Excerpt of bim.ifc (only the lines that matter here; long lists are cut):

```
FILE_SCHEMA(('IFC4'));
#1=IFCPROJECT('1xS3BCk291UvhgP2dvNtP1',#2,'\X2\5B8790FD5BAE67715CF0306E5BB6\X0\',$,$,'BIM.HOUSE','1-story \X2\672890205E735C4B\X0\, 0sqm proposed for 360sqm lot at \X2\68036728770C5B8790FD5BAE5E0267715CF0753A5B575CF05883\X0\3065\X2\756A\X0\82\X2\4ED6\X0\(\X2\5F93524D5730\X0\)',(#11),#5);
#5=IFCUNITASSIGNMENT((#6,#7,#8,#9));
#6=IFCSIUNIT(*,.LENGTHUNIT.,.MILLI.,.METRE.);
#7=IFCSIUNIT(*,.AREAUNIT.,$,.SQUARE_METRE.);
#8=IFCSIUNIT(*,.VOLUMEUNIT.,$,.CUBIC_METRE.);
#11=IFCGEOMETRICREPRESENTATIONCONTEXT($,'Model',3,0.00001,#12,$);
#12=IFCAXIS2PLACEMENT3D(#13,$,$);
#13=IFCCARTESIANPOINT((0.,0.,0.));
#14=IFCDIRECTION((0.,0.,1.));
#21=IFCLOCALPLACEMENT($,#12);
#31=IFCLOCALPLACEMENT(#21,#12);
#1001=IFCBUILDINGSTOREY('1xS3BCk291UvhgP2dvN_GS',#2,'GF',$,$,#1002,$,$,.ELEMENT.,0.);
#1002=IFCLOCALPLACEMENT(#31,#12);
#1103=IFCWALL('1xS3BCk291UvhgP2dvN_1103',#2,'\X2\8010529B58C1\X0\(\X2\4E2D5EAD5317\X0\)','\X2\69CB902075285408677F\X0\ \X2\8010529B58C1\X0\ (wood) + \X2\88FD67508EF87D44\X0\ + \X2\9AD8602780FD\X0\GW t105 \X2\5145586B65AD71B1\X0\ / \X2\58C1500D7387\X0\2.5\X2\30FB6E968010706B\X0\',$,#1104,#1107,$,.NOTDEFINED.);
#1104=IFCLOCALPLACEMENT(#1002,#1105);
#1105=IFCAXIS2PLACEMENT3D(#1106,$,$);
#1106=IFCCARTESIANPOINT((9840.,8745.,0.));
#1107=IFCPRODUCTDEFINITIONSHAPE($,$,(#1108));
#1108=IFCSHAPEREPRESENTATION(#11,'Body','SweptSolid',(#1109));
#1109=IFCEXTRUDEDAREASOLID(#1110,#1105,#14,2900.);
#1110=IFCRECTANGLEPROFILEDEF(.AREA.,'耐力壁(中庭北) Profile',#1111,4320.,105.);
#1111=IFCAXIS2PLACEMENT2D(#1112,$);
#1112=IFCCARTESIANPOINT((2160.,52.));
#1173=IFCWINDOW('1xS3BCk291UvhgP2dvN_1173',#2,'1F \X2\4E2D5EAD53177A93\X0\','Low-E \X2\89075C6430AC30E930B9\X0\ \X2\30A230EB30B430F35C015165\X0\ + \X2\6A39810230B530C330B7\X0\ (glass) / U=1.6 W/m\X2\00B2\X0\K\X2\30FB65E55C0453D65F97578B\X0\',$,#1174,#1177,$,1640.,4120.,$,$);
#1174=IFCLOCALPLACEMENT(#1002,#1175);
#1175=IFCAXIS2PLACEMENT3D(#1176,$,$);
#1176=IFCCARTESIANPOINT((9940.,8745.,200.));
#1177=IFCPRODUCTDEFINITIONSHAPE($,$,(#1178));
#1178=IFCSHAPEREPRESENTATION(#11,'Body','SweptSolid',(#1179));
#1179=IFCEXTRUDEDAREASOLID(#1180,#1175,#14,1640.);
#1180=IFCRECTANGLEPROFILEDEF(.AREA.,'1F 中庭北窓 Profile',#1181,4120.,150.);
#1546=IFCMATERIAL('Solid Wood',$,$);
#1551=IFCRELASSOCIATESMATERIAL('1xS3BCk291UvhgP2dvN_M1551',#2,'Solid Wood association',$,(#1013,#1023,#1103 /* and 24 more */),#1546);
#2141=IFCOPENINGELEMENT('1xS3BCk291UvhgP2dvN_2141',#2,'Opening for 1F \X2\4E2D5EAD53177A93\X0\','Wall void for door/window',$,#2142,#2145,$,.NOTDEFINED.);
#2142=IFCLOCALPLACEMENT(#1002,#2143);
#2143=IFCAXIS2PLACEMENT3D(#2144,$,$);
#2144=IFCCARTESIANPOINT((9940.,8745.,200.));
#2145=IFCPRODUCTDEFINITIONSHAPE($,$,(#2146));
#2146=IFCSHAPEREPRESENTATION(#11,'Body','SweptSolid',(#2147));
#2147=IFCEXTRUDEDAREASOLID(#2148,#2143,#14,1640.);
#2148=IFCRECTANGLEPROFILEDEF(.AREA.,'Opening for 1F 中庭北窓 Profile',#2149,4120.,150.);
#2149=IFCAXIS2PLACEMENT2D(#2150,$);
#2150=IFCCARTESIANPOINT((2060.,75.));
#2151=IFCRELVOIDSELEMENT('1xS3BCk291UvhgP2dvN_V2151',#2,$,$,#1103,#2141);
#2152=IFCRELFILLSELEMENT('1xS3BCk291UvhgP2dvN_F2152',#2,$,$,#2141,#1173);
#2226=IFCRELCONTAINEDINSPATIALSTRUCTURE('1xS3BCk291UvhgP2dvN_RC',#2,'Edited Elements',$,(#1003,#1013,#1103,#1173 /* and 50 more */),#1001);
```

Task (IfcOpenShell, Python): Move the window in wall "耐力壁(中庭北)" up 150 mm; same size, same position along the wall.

```python
import numpy as np
import ifcopenshell
import ifcopenshell.api.geometry
import ifcopenshell.util.placement
import ifcopenshell.util.unit

model = ifcopenshell.open("bim.ifc")
unit_scale = ifcopenshell.util.unit.calculate_unit_scale(model)

window = model.by_guid("1xS3BCk291UvhgP2dvN_1173")
opening = window.FillsVoids[0].RelatingOpeningElement
dz = 0.15 / unit_scale

shift = np.array([0.0, 0.0, dz])
# The window is not placed relative to its opening, so move both.
for product in (opening, window):
    matrix = ifcopenshell.util.placement.get_local_placement(product.ObjectPlacement)
    matrix[:3, 3] += shift
    ifcopenshell.api.geometry.edit_object_placement(model, product=product, matrix=matrix, is_si=False)

print(f"moved by {dz * unit_scale:+.3f} m")

model.write("bim_updated.ifc")
```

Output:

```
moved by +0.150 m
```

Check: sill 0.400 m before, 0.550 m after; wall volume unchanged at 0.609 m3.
